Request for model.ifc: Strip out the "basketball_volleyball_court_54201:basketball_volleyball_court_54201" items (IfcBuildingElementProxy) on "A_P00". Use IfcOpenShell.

First a look at what the model holds.

```python
import ifcopenshell
import ifcopenshell.util.element

model = ifcopenshell.open("model.ifc")
print(model.schema)
storey = next(s for s in model.by_type("IfcBuildingStorey") if s.Name == "A_P00")
proxies = [e for e in ifcopenshell.util.element.get_decomposition(storey) if e.is_a("IfcBuildingElementProxy")]
seen = {}
for e in proxies:
    element_type = ifcopenshell.util.element.get_type(e)
    name = element_type.Name if element_type not in (None, e) else None
    seen[name] = seen.get(name, 0) + 1
for name, count in sorted(seen.items(), key=str):
    print(count, "x", name)
```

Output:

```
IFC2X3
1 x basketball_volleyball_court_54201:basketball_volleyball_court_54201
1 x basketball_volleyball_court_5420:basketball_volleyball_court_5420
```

```python
import ifcopenshell
import ifcopenshell.api.root
import ifcopenshell.util.element

model = ifcopenshell.open("model.ifc")

storey = next(s for s in model.by_type("IfcBuildingStorey") if s.Name == "A_P00")
proxies = [e for e in ifcopenshell.util.element.get_decomposition(storey) if e.is_a("IfcBuildingElementProxy")]
targets = [e for e in proxies if (t := ifcopenshell.util.element.get_type(e)) not in (None, e) and t.Name == "basketball_volleyball_court_54201:basketball_volleyball_court_54201"]

for e in targets:
    ifcopenshell.api.root.remove_product(model, product=e)
print(len(targets), "removed")

model.write("model_rev.ifc")
```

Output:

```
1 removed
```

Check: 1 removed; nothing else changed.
